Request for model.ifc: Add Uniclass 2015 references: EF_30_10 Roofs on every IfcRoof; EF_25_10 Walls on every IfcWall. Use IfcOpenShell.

First a look at what the model holds.

```python
import ifcopenshell

model = ifcopenshell.open("model.ifc")
print(model.schema)
print("classifications:", [c.Name for c in model.by_type("IfcClassification")])
for ifc_class in ("IfcDoor", "IfcRoof", "IfcStair", "IfcWall", "IfcWindow"):
    print(ifc_class, len(model.by_type(ifc_class)))
```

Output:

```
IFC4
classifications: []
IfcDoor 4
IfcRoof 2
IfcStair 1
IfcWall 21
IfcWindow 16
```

```python
import ifcopenshell
import ifcopenshell.api.classification

model = ifcopenshell.open("model.ifc")

system = ifcopenshell.api.classification.add_classification(model, classification="Uniclass 2015")

codes = {
    "IfcRoof": ("EF_30_10", "Roofs"),
    "IfcWall": ("EF_25_10", "Walls"),
}
for ifc_class, (code, name) in codes.items():
    products = model.by_type(ifc_class)
    ifcopenshell.api.classification.add_reference(
        model, products=products, classification=system, identification=code, name=name
    )
    print(code, len(products))

model.write("model_updated.ifc")
```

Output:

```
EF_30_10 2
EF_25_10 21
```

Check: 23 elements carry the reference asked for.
